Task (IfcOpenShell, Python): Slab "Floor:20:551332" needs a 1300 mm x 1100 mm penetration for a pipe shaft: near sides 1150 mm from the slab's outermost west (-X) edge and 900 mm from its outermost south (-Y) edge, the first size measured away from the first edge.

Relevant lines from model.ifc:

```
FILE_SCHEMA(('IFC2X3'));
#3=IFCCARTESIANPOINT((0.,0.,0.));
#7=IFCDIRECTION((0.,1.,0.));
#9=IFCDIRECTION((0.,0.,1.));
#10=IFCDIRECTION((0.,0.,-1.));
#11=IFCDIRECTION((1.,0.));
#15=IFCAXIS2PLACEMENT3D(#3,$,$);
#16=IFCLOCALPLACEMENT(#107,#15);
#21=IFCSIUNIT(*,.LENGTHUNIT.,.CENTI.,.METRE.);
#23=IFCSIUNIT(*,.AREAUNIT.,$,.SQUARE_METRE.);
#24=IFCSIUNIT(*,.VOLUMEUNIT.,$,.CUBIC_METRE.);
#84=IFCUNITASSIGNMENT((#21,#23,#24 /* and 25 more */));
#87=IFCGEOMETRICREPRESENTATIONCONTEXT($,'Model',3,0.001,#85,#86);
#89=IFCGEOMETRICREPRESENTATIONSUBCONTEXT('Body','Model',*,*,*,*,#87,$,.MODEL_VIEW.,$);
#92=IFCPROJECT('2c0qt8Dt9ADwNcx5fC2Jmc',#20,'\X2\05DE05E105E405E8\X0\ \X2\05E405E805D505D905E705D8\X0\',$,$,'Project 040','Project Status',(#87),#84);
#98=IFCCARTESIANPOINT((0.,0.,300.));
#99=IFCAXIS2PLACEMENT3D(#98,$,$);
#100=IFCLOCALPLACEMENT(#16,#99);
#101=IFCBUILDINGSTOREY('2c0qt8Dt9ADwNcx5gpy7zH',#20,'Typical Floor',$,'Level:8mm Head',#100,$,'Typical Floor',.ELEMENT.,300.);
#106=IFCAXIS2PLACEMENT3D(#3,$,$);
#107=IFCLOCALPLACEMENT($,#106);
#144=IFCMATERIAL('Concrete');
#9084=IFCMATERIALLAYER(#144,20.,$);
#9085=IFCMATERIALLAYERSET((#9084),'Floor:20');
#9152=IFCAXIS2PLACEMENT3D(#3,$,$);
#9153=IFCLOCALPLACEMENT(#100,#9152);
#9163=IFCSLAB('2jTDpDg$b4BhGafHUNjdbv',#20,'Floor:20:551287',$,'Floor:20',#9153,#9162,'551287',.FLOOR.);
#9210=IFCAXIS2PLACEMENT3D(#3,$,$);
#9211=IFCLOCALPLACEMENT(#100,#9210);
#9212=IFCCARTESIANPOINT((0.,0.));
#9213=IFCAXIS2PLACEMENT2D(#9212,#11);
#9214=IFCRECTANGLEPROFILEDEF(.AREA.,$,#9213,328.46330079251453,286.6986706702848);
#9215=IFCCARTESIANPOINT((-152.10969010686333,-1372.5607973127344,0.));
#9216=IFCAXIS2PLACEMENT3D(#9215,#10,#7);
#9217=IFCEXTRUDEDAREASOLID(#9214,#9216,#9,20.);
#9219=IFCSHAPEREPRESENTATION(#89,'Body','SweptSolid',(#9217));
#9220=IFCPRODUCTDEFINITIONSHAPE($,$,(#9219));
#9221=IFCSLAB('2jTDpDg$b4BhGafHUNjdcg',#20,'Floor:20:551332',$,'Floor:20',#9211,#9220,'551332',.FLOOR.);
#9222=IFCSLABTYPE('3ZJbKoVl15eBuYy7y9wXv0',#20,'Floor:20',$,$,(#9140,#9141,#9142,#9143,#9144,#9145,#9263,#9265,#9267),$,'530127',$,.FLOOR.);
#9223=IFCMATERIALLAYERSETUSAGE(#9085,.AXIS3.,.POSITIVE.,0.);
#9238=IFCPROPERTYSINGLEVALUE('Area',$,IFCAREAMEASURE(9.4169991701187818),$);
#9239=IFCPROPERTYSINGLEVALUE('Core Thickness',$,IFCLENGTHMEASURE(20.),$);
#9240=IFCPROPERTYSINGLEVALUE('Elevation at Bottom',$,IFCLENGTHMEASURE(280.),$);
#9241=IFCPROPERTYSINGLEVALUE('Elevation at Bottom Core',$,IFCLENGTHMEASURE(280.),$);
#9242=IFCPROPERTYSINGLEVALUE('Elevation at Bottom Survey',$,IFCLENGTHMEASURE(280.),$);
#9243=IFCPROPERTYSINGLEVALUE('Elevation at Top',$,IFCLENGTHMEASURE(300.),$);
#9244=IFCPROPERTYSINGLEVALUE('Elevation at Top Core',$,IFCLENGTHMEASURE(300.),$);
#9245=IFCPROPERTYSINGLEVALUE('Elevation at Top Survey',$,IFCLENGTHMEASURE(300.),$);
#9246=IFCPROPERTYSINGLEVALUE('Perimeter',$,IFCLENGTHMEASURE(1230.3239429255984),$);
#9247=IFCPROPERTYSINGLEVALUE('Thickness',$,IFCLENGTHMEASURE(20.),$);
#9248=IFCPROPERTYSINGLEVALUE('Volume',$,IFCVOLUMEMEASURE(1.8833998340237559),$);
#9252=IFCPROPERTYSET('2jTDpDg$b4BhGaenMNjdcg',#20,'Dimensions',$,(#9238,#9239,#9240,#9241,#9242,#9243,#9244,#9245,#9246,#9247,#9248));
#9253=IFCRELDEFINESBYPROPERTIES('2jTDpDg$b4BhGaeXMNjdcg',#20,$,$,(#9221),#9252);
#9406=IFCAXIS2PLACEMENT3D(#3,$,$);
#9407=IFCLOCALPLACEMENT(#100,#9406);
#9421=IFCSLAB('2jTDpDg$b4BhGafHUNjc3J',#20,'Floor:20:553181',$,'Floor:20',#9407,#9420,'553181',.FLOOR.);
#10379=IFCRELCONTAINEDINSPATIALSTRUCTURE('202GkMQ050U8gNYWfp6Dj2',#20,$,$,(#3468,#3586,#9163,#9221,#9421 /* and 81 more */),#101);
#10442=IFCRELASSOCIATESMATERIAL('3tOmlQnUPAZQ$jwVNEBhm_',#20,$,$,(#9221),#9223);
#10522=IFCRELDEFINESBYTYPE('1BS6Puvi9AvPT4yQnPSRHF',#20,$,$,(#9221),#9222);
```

```python
import numpy as np
import ifcopenshell
import ifcopenshell.api.feature
import ifcopenshell.api.geometry
import ifcopenshell.api.pset
import ifcopenshell.api.root
import ifcopenshell.geom
import ifcopenshell.util.element
import ifcopenshell.util.placement
import ifcopenshell.util.representation
import ifcopenshell.util.shape
import ifcopenshell.util.unit

model = ifcopenshell.open("model.ifc")
unit_scale = ifcopenshell.util.unit.calculate_unit_scale(model)
area_scale = ifcopenshell.util.unit.calculate_unit_scale(model, "AREAUNIT")
volume_scale = ifcopenshell.util.unit.calculate_unit_scale(model, "VOLUMEUNIT")
settings = ifcopenshell.geom.settings()


def volume(element):
    """Net volume in cubic metres, openings subtracted."""
    shape = ifcopenshell.geom.create_shape(settings, element)
    return ifcopenshell.util.shape.get_volume(shape.geometry)


slab = model.by_guid("2jTDpDg$b4BhGafHUNjdcg")
before = volume(slab)

# Extent in the slab's own axes, in metres. The edges named are its -X and -Y sides.
slab_shape = ifcopenshell.geom.create_shape(settings, slab)
vertices = ifcopenshell.util.shape.get_vertices(slab_shape.geometry)
x_min, y_min, bottom = vertices.min(axis=0)
top = vertices[:, 2].max()

opening = ifcopenshell.api.root.create_entity(model, ifc_class="IfcOpeningElement", name="Pipe shaft opening")
context = ifcopenshell.util.representation.get_context(model, "Model", "Body", "MODEL_VIEW")
width, depth = 1.3, 1.1
outline = [(0.0, 0.0), (width, 0.0), (width, depth), (0.0, depth), (0.0, 0.0)]
# Overshoot both faces by 50 mm so the cut is clean.
shape = ifcopenshell.api.geometry.add_slab_representation(
    model, context=context, depth=top - bottom + 0.1, polyline=outline
)
ifcopenshell.api.geometry.assign_representation(model, product=opening, representation=shape)

matrix = ifcopenshell.util.placement.get_local_placement(slab.ObjectPlacement)
matrix[:, 3] = matrix @ np.append(np.array([x_min + 1.15, y_min + 0.9, bottom - 0.05]) / unit_scale, 1.0)
ifcopenshell.api.geometry.edit_object_placement(model, product=opening, matrix=matrix, is_si=False)
ifcopenshell.api.feature.add_feature(model, feature=opening, element=slab)

after = volume(slab)

# Update the slab's stored quantities.
pset = model.by_id(ifcopenshell.util.element.get_pset(slab, "Dimensions", should_inherit=False)["id"])
ifcopenshell.api.pset.edit_pset(model, pset=pset, properties={
    "Area": model.create_entity("IfcAreaMeasure", after / (top - bottom) / area_scale),
    "Volume": model.create_entity("IfcVolumeMeasure", after / volume_scale),
})

print(f"slab volume {before:.3f} -> {after:.3f} m3")

model.write("model-out.ifc")
```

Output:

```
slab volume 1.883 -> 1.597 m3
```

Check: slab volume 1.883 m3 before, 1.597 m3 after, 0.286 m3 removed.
